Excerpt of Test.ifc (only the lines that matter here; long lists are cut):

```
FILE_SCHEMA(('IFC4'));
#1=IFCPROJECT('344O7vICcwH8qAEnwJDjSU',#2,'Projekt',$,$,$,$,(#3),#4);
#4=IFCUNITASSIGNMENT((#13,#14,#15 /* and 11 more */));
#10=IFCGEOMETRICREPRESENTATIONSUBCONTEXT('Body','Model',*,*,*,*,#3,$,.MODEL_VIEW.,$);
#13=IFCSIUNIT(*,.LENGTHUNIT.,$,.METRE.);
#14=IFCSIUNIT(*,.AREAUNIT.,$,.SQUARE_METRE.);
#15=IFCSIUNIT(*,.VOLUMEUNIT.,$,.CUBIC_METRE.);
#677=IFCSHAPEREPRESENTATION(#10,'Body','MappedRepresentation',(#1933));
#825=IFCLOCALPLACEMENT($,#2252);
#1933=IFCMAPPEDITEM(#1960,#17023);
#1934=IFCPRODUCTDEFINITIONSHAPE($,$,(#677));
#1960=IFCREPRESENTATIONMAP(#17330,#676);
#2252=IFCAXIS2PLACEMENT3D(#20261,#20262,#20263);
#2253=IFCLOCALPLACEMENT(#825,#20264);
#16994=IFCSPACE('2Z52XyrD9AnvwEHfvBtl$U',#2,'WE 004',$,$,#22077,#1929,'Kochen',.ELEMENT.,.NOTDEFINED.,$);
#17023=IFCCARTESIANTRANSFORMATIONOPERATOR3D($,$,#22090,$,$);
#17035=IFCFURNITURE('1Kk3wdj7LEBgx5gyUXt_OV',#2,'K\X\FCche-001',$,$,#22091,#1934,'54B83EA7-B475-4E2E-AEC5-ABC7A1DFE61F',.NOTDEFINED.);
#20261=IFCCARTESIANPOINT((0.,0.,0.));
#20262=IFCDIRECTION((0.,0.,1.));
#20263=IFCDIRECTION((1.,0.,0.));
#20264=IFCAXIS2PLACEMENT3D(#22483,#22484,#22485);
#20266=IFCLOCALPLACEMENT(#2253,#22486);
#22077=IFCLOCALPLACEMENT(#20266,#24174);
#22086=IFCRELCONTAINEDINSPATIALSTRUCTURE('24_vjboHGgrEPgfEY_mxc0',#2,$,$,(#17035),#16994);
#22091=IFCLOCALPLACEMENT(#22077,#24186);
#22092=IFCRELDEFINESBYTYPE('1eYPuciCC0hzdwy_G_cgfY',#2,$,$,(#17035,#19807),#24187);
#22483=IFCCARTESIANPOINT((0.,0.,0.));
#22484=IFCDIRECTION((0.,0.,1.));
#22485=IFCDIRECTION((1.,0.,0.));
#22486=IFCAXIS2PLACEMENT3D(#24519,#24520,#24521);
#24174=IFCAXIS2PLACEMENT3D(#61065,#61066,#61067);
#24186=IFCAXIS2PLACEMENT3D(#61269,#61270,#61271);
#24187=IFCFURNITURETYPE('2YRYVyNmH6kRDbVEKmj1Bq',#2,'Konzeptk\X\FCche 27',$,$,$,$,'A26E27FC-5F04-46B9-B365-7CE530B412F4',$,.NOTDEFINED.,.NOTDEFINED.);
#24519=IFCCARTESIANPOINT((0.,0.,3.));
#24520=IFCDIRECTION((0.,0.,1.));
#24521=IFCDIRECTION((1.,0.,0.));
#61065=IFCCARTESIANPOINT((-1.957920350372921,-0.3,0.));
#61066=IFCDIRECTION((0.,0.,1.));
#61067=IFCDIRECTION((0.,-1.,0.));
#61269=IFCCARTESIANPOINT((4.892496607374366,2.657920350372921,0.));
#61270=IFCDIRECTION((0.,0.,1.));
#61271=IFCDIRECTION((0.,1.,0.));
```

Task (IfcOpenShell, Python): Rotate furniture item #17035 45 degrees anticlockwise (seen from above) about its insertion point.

```python
import ifcopenshell
import ifcopenshell.api.geometry
import ifcopenshell.util.placement

model = ifcopenshell.open("Test.ifc")

item = model.by_guid("1Kk3wdj7LEBgx5gyUXt_OV")
matrix = ifcopenshell.util.placement.get_local_placement(item.ObjectPlacement)
matrix = matrix @ ifcopenshell.util.placement.rotation(45, "Z")
ifcopenshell.api.geometry.edit_object_placement(model, product=item, matrix=matrix, is_si=False)

print(ifcopenshell.util.placement.get_local_placement(item.ObjectPlacement).round(3) + 0.0)

model.write("Test-out.ifc")
```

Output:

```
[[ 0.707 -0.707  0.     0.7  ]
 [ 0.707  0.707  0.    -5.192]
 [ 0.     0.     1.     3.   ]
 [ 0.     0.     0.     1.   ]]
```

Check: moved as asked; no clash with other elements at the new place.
